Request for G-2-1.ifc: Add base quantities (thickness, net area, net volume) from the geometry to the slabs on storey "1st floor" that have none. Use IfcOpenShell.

First a look at what the model holds.

```python
import ifcopenshell
import ifcopenshell.util.element
import ifcopenshell.util.unit

model = ifcopenshell.open("G-2-1.ifc")
print(model.schema)
for unit_type in ("LENGTHUNIT", "AREAUNIT", "VOLUMEUNIT"):
    print(unit_type, ifcopenshell.util.unit.calculate_unit_scale(model, unit_type))
storey = next(s for s in model.by_type("IfcBuildingStorey") if s.Name == "1st floor")
slabs = [e for e in ifcopenshell.util.element.get_decomposition(storey) if e.is_a("IfcSlab")]
for e in sorted(slabs, key=lambda e: e.id()):
    print(e.id(), e.is_a(), e.Name, list(ifcopenshell.util.element.get_psets(e, qtos_only=True)), sep=" | ")
```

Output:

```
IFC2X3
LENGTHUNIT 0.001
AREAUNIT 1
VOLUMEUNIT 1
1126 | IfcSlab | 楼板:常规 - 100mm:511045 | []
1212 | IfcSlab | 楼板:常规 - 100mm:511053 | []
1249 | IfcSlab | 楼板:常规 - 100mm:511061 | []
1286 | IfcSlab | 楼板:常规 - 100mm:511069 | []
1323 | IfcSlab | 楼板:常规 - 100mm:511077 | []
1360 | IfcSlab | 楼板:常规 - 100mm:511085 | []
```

```python
import ifcopenshell
import ifcopenshell.api.pset
import ifcopenshell.geom
import ifcopenshell.util.element
import ifcopenshell.util.shape
import ifcopenshell.util.unit

model = ifcopenshell.open("G-2-1.ifc")
unit_scale = ifcopenshell.util.unit.calculate_unit_scale(model)
area_scale = ifcopenshell.util.unit.calculate_unit_scale(model, "AREAUNIT")
volume_scale = ifcopenshell.util.unit.calculate_unit_scale(model, "VOLUMEUNIT")
settings = ifcopenshell.geom.settings()

storey = next(s for s in model.by_type("IfcBuildingStorey") if s.Name == "1st floor")
slabs = [e for e in ifcopenshell.util.element.get_decomposition(storey) if e.is_a("IfcSlab")]

for e in sorted(slabs, key=lambda e: e.id()):
    if ifcopenshell.util.element.get_psets(e, qtos_only=True, should_inherit=False):
        continue
    # Geometry comes back in metres, in the element's own axes.
    shape = ifcopenshell.geom.create_shape(settings, e)
    values = {
        "Width": ifcopenshell.util.shape.get_z(shape.geometry) / unit_scale,
        "NetArea": ifcopenshell.util.shape.get_footprint_area(shape.geometry) / area_scale,
        "NetVolume": ifcopenshell.util.shape.get_volume(shape.geometry) / volume_scale,
    }
    qto = ifcopenshell.api.pset.add_qto(model, product=e, name="BaseQuantities")
    ifcopenshell.api.pset.edit_qto(model, qto=qto, properties=values)
    print(e.id(), {k: round(v, 3) for k, v in values.items()})

model.write("G-2-1-out.ifc")
```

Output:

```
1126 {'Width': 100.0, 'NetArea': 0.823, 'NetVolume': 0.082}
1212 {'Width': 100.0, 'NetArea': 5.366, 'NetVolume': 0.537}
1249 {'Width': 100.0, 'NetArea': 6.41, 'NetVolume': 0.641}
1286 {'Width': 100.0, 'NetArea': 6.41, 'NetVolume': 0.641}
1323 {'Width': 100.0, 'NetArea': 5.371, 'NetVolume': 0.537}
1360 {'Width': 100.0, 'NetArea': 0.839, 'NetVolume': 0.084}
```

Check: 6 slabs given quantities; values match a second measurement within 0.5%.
